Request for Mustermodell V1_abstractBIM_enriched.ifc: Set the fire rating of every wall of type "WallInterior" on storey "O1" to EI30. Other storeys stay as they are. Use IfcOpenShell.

First a look at what the model holds.

```python
import ifcopenshell
import ifcopenshell.util.element

model = ifcopenshell.open("Mustermodell V1_abstractBIM_enriched.ifc")
print(model.schema)
storey = next(s for s in model.by_type("IfcBuildingStorey") if s.Name == "O1")
walls = [e for e in ifcopenshell.util.element.get_decomposition(storey) if e.is_a("IfcWall")]
seen = {}
for e in walls:
    element_type = ifcopenshell.util.element.get_type(e)
    key = (element_type.Name if element_type != e and element_type else None, ifcopenshell.util.element.get_pset(e, "Pset_WallCommon", "FireRating"))
    seen[key] = seen.get(key, 0) + 1
for (name, value), count in sorted(seen.items(), key=str):
    print(count, "x", name, "|", value)
```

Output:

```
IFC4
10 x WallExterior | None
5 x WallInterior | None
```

```python
import ifcopenshell
import ifcopenshell.api.pset
import ifcopenshell.util.element

model = ifcopenshell.open("Mustermodell V1_abstractBIM_enriched.ifc")

storey = next(s for s in model.by_type("IfcBuildingStorey") if s.Name == "O1")
walls = [e for e in ifcopenshell.util.element.get_decomposition(storey) if e.is_a("IfcWall")]

count = 0
for e in walls:
    element_type = ifcopenshell.util.element.get_type(e)
    if element_type in (None, e) or element_type.Name != "WallInterior":
        continue
    # add_pset returns the element's existing set when there is one.
    pset = ifcopenshell.api.pset.add_pset(model, product=e, name="Pset_WallCommon")
    ifcopenshell.api.pset.edit_pset(model, pset=pset, properties={"FireRating": "EI30"})
    count += 1

print(count, "walls updated")

model.write("Mustermodell V1_abstractBIM_enriched_edited.ifc")
```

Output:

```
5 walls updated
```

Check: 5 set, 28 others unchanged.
